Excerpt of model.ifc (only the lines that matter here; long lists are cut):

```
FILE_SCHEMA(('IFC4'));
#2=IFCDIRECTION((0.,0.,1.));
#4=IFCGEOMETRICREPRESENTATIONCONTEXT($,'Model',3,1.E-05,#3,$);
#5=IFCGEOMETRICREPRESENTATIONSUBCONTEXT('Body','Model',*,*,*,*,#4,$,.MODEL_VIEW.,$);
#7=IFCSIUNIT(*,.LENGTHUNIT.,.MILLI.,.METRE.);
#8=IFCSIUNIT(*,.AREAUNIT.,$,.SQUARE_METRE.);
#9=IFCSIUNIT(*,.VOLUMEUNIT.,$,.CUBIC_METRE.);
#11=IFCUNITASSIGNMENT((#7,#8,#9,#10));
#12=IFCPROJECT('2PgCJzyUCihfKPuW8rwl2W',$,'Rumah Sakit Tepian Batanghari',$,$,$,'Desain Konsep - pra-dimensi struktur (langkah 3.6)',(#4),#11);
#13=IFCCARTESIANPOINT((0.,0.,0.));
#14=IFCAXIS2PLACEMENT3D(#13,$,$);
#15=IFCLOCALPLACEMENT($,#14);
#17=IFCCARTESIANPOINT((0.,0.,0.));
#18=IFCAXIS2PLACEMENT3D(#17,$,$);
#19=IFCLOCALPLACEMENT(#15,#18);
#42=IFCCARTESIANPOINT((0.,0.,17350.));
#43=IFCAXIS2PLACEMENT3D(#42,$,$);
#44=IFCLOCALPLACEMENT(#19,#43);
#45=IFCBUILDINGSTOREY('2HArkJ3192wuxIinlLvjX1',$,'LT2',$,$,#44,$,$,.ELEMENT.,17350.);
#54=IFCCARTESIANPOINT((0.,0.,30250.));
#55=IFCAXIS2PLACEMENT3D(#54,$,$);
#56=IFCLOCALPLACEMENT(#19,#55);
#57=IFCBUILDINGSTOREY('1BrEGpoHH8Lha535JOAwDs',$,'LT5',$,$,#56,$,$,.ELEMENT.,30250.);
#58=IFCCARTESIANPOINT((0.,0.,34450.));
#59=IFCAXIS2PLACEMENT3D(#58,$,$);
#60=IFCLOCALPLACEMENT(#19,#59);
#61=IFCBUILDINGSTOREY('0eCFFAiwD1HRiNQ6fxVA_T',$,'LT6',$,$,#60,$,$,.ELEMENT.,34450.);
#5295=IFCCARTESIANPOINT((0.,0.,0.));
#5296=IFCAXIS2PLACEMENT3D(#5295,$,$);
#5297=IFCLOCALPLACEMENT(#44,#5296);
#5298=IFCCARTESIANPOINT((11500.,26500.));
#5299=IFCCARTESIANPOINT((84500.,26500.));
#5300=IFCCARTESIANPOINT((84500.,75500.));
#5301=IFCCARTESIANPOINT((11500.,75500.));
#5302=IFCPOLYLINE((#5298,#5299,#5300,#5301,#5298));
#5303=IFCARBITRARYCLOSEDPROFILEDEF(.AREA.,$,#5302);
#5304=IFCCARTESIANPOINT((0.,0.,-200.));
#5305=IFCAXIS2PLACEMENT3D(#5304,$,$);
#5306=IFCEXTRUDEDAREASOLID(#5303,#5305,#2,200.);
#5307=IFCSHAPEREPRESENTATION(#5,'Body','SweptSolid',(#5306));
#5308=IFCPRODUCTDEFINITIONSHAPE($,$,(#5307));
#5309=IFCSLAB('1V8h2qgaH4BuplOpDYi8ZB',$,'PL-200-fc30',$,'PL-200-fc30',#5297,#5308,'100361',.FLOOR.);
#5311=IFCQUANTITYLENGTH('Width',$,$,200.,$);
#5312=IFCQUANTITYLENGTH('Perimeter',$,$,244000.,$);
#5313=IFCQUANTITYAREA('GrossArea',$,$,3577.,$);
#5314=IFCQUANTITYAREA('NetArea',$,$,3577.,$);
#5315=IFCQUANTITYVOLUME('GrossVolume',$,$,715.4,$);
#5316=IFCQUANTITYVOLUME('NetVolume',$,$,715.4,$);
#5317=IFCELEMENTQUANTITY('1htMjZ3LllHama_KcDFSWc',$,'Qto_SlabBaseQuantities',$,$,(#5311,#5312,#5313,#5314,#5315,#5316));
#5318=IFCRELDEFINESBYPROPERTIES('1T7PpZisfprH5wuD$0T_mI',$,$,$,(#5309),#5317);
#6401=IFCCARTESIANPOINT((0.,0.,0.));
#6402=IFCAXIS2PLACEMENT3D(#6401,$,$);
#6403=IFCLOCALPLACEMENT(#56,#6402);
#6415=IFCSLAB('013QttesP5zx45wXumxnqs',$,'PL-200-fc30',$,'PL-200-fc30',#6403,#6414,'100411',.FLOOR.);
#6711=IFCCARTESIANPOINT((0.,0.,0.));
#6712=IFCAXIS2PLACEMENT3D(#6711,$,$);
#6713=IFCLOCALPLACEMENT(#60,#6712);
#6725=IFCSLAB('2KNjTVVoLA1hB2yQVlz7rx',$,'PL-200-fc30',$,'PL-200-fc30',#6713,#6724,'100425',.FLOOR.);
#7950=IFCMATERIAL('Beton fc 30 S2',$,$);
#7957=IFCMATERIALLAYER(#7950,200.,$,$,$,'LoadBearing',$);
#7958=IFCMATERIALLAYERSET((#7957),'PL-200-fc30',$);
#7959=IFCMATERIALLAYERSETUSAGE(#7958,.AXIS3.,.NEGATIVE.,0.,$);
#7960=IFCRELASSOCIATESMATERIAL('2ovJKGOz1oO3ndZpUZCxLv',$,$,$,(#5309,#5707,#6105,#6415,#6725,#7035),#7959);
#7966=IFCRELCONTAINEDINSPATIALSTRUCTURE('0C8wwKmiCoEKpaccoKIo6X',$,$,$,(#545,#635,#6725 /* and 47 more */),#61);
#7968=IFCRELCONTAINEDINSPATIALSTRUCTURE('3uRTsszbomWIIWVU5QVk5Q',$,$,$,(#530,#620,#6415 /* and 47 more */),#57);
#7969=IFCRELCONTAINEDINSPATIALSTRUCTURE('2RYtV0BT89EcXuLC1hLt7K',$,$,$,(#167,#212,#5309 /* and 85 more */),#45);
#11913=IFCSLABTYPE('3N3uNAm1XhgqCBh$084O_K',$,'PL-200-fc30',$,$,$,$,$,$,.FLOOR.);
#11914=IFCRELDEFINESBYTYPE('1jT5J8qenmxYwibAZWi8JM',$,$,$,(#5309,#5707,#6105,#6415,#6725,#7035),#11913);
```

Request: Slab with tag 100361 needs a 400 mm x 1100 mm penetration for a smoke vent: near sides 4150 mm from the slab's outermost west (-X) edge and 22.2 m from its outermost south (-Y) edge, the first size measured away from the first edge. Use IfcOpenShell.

```python
import numpy as np
import ifcopenshell
import ifcopenshell.api.feature
import ifcopenshell.api.geometry
import ifcopenshell.api.pset
import ifcopenshell.api.root
import ifcopenshell.geom
import ifcopenshell.util.element
import ifcopenshell.util.placement
import ifcopenshell.util.representation
import ifcopenshell.util.shape
import ifcopenshell.util.unit

model = ifcopenshell.open("model.ifc")
unit_scale = ifcopenshell.util.unit.calculate_unit_scale(model)
area_scale = ifcopenshell.util.unit.calculate_unit_scale(model, "AREAUNIT")
volume_scale = ifcopenshell.util.unit.calculate_unit_scale(model, "VOLUMEUNIT")
settings = ifcopenshell.geom.settings()


def volume(element):
    """Net volume in cubic metres, openings subtracted."""
    shape = ifcopenshell.geom.create_shape(settings, element)
    return ifcopenshell.util.shape.get_volume(shape.geometry)


slab = model.by_guid("1V8h2qgaH4BuplOpDYi8ZB")
before = volume(slab)

# Extent in the slab's own axes, in metres. The edges named are its -X and -Y sides.
slab_shape = ifcopenshell.geom.create_shape(settings, slab)
vertices = ifcopenshell.util.shape.get_vertices(slab_shape.geometry)
x_min, y_min, bottom = vertices.min(axis=0)
top = vertices[:, 2].max()

opening = ifcopenshell.api.root.create_entity(model, ifc_class="IfcOpeningElement", name="Smoke vent opening", predefined_type="OPENING")
context = ifcopenshell.util.representation.get_context(model, "Model", "Body", "MODEL_VIEW")
width, depth = 0.4, 1.1
outline = [(0.0, 0.0), (width, 0.0), (width, depth), (0.0, depth), (0.0, 0.0)]
# Overshoot both faces by 50 mm so the cut is clean.
shape = ifcopenshell.api.geometry.add_slab_representation(
    model, context=context, depth=top - bottom + 0.1, polyline=outline
)
ifcopenshell.api.geometry.assign_representation(model, product=opening, representation=shape)

matrix = ifcopenshell.util.placement.get_local_placement(slab.ObjectPlacement)
matrix[:, 3] = matrix @ np.append(np.array([x_min + 4.15, y_min + 22.2, bottom - 0.05]) / unit_scale, 1.0)
ifcopenshell.api.geometry.edit_object_placement(model, product=opening, matrix=matrix, is_si=False)
ifcopenshell.api.feature.add_feature(model, feature=opening, element=slab)

after = volume(slab)

# Update the slab's stored quantities.
qto = model.by_id(ifcopenshell.util.element.get_pset(slab, "Qto_SlabBaseQuantities", should_inherit=False)["id"])
ifcopenshell.api.pset.edit_qto(model, qto=qto, properties={
    "NetArea": after / (top - bottom) / area_scale,
    "NetVolume": after / volume_scale,
})

print(f"slab volume {before:.3f} -> {after:.3f} m3")

model.write("model_v2.ifc")
```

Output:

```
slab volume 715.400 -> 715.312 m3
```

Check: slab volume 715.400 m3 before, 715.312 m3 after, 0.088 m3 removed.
